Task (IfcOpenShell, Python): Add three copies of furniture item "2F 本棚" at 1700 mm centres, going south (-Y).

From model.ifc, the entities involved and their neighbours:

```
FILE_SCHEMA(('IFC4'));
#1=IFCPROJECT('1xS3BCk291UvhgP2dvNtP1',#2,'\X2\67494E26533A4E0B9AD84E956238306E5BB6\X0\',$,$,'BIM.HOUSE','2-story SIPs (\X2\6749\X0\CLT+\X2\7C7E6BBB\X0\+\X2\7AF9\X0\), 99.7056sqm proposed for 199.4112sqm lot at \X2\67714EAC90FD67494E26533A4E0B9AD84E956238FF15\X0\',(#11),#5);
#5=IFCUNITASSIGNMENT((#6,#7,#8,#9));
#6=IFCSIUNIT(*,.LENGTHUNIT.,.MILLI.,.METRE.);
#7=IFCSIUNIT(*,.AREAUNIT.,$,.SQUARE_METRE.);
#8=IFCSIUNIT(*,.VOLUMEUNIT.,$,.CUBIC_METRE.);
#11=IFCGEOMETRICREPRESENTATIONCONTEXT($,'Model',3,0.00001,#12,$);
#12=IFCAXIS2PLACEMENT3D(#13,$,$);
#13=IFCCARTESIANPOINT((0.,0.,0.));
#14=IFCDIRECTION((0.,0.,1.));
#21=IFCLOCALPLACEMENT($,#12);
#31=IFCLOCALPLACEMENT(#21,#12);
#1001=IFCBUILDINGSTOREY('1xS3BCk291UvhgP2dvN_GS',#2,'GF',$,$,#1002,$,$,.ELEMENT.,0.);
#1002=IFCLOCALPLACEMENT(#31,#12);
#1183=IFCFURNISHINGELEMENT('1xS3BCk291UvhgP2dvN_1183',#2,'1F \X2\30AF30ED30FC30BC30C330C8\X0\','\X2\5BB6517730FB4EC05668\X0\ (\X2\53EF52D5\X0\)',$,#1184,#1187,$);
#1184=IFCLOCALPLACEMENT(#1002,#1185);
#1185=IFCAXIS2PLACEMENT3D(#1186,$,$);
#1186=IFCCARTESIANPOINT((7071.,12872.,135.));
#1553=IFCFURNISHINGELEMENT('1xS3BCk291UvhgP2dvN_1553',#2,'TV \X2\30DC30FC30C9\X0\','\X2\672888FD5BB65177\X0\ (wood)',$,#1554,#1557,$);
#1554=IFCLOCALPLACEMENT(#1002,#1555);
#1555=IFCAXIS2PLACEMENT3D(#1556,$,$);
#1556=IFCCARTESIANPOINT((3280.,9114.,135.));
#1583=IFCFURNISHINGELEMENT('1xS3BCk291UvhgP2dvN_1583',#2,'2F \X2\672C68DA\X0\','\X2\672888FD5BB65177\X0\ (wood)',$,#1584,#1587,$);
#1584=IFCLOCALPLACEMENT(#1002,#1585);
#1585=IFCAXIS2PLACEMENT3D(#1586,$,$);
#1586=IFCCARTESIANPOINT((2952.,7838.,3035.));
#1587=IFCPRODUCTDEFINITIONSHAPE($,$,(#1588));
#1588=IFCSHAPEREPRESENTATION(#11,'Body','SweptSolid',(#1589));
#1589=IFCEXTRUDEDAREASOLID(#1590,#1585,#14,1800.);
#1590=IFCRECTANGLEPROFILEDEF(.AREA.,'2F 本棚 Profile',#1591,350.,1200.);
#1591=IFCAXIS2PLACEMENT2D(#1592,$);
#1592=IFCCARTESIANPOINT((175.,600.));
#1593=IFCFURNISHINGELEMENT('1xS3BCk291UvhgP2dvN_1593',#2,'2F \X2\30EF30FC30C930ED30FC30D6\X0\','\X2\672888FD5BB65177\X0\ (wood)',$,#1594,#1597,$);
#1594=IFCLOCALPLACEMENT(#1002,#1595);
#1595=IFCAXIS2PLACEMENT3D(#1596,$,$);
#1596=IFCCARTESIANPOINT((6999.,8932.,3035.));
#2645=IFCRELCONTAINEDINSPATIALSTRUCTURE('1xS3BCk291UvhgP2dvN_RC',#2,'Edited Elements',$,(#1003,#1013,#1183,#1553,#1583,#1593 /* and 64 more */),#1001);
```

```python
import numpy as np
import ifcopenshell
import ifcopenshell.api.geometry
import ifcopenshell.api.root
import ifcopenshell.util.element
import ifcopenshell.util.placement
import ifcopenshell.util.unit

model = ifcopenshell.open("model.ifc")
unit_scale = ifcopenshell.util.unit.calculate_unit_scale(model)


def reuse_history(source, copy):
    """copy_class also copies each property set's owner history, people and application; keep the originals."""
    for rel in copy.IsDefinedBy:
        if rel.is_a("IfcRelDefinesByProperties") and (history := rel.RelatingPropertyDefinition.OwnerHistory):
            rel.RelatingPropertyDefinition.OwnerHistory = source.OwnerHistory
            ifcopenshell.util.element.remove_deep2(model, history)


source = model.by_guid("1xS3BCk291UvhgP2dvN_1583")
base = ifcopenshell.util.placement.get_local_placement(source.ObjectPlacement)
step = np.array([0.0, -1.0, 0.0]) * 1.7 / unit_scale

for i in range(1, 4):
    copy = ifcopenshell.api.root.copy_class(model, product=source)
    copy.Representation = ifcopenshell.util.element.copy_deep(
        model, source.Representation, exclude=["IfcGeometricRepresentationContext", "IfcRepresentationMap"]
    )
    reuse_history(source, copy)
    matrix = base.copy()
    matrix[:3, 3] += i * step
    print("added at", matrix[:3, 3].round(3) + 0.0)
    ifcopenshell.api.geometry.edit_object_placement(model, product=copy, matrix=matrix, is_si=False)

model.write("model_edited.ifc")
```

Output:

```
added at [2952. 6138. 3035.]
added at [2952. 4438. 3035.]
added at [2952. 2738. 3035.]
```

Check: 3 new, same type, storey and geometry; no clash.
